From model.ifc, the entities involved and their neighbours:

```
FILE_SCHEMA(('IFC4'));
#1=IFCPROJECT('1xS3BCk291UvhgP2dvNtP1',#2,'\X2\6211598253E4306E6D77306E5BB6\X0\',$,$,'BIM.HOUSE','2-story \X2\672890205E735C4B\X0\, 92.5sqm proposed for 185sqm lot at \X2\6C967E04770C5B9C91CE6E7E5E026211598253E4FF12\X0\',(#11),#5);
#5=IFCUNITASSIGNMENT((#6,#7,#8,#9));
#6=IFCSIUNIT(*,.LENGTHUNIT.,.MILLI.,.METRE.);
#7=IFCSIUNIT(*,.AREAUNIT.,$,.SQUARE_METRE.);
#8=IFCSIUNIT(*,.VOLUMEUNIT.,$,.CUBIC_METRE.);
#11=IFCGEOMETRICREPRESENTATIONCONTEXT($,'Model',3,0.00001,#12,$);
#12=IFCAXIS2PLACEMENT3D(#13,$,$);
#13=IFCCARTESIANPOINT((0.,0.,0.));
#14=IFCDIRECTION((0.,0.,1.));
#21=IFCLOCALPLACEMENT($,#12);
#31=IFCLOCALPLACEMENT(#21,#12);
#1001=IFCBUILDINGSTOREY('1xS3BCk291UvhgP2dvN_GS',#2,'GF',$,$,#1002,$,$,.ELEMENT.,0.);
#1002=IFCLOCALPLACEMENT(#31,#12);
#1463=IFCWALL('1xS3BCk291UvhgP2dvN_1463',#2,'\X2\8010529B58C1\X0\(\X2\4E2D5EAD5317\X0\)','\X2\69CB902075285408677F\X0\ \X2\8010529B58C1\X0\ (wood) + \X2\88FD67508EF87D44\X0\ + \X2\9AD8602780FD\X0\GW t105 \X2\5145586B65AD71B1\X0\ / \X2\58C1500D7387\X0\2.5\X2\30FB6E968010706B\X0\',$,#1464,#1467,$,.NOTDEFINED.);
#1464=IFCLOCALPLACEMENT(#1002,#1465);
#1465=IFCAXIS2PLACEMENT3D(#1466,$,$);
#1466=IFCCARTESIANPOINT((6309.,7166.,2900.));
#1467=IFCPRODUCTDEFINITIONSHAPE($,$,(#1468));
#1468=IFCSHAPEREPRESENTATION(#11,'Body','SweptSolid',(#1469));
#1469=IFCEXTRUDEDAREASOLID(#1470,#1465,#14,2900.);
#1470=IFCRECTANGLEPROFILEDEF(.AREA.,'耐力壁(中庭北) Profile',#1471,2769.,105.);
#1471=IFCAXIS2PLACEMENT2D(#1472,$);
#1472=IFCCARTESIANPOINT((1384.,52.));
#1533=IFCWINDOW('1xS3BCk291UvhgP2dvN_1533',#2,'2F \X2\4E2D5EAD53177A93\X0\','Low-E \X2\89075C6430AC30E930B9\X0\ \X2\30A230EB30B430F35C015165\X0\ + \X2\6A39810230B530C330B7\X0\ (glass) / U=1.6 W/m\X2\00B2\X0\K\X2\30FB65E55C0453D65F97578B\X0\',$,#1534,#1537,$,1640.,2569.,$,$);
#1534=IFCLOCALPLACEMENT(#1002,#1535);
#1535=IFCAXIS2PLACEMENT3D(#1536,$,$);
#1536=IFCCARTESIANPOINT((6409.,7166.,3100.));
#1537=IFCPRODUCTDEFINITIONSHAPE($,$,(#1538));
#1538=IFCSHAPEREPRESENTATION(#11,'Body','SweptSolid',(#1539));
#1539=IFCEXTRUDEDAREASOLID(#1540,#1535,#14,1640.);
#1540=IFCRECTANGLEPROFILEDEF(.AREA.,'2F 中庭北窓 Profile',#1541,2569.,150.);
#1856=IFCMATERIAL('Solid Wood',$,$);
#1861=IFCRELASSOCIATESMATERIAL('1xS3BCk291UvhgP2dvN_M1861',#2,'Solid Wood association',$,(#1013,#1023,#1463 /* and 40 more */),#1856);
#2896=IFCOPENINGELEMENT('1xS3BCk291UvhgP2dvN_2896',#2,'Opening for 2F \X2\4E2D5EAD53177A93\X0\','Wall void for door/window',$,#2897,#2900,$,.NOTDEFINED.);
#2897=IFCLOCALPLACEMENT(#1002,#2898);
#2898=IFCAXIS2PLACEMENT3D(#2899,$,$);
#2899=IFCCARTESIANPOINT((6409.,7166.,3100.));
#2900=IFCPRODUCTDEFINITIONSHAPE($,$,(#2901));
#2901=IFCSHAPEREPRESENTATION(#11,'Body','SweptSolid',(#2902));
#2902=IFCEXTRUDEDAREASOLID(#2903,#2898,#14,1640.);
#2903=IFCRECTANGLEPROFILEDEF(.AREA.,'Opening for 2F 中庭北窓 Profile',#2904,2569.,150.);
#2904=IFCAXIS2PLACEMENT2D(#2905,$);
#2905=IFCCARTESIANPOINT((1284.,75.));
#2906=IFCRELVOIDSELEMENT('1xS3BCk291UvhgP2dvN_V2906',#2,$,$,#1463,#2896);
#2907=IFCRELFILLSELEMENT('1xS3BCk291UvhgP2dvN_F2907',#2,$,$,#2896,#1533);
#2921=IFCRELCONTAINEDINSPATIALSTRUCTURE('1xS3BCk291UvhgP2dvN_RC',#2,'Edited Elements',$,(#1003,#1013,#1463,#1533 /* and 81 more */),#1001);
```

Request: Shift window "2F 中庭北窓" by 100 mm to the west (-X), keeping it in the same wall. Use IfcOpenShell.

```python
import ifcopenshell
import ifcopenshell.api.geometry
import ifcopenshell.util.placement
import ifcopenshell.util.unit

model = ifcopenshell.open("model.ifc")
unit_scale = ifcopenshell.util.unit.calculate_unit_scale(model)

window = model.by_guid("1xS3BCk291UvhgP2dvN_1533")
opening = window.FillsVoids[0].RelatingOpeningElement
wall = opening.VoidsElements[0].RelatingBuildingElement

wall_matrix = ifcopenshell.util.placement.get_local_placement(wall.ObjectPlacement)
shift = wall_matrix[:3, 0] * -0.1 / unit_scale
before = ifcopenshell.util.placement.get_local_placement(window.ObjectPlacement)[:3, 3].copy()

# The window is not placed relative to its opening, so move both.
for product in (opening, window):
    matrix = ifcopenshell.util.placement.get_local_placement(product.ObjectPlacement)
    matrix[:3, 3] += shift
    ifcopenshell.api.geometry.edit_object_placement(model, product=product, matrix=matrix, is_si=False)

after = ifcopenshell.util.placement.get_local_placement(window.ObjectPlacement)[:3, 3]
print("window moved by", (after - before).round(3) + 0.0)

model.write("model_rev.ifc")
```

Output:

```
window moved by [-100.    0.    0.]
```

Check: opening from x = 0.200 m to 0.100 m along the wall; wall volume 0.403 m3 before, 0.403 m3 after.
